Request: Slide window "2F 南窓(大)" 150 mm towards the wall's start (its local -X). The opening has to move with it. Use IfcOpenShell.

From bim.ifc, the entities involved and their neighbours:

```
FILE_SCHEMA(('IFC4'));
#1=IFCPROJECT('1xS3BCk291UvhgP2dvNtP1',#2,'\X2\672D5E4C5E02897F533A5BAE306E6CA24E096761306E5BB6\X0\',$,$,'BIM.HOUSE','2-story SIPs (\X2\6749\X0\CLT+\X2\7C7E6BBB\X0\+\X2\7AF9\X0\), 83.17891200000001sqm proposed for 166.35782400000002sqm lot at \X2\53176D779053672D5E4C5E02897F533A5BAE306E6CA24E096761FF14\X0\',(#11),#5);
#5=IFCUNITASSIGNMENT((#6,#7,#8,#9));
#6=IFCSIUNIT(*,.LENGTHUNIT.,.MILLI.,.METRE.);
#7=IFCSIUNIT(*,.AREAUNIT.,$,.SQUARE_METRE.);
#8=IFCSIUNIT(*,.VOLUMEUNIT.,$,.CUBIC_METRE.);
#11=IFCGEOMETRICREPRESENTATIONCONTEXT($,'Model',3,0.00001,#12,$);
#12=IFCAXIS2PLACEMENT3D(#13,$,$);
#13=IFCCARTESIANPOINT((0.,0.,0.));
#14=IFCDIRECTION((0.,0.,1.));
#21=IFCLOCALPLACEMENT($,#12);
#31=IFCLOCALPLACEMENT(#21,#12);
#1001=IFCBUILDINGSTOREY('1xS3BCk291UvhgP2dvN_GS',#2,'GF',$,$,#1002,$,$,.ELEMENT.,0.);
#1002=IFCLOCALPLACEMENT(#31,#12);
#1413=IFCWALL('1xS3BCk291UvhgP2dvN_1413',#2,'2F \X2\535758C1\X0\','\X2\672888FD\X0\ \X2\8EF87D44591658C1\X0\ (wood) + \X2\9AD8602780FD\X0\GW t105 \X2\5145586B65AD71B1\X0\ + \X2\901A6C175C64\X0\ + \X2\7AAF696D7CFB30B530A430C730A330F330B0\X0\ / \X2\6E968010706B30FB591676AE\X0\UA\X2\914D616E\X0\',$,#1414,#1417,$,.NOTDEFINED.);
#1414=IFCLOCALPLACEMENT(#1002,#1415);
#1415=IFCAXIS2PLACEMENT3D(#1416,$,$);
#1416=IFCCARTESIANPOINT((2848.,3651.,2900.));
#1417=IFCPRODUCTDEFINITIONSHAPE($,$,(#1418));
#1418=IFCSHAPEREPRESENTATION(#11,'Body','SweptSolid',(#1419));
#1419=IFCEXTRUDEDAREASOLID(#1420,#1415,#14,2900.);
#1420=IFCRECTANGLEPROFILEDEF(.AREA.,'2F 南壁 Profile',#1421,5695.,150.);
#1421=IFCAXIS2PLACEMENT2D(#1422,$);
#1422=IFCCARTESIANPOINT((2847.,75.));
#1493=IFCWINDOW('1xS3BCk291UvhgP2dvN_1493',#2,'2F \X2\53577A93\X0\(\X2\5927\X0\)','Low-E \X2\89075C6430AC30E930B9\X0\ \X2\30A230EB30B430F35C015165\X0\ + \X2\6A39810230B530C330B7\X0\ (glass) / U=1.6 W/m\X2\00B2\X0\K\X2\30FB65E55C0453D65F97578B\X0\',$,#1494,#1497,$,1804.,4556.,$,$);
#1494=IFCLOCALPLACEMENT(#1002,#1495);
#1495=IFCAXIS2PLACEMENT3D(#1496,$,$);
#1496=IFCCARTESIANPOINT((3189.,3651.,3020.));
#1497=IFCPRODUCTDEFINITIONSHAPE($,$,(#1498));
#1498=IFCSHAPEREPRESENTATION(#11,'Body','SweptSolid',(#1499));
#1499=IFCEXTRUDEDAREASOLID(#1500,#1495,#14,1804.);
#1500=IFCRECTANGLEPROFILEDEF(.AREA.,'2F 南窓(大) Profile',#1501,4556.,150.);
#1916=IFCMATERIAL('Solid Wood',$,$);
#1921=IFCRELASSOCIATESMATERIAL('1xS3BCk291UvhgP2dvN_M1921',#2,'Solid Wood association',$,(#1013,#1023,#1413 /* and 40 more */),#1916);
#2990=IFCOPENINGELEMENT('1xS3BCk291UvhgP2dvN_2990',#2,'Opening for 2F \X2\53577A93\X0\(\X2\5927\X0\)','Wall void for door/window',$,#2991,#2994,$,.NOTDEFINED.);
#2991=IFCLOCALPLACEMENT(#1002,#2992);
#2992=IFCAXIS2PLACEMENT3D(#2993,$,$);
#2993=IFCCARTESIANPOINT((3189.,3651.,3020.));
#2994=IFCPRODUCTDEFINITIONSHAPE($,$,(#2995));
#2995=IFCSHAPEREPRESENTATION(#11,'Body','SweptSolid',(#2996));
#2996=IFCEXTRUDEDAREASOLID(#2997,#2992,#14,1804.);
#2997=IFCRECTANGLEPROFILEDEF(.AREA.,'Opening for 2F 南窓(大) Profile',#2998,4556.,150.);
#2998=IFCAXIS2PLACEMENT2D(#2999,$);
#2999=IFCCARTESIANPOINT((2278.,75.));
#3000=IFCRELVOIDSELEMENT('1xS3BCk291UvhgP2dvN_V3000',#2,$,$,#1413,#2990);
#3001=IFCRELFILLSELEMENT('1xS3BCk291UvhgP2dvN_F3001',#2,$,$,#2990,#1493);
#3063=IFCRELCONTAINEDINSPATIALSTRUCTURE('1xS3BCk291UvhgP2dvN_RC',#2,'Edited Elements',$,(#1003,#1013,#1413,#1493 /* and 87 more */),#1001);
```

```python
import ifcopenshell
import ifcopenshell.api.geometry
import ifcopenshell.util.placement
import ifcopenshell.util.unit

model = ifcopenshell.open("bim.ifc")
unit_scale = ifcopenshell.util.unit.calculate_unit_scale(model)

window = model.by_guid("1xS3BCk291UvhgP2dvN_1493")
opening = window.FillsVoids[0].RelatingOpeningElement
wall = opening.VoidsElements[0].RelatingBuildingElement

wall_matrix = ifcopenshell.util.placement.get_local_placement(wall.ObjectPlacement)
shift = wall_matrix[:3, 0] * -0.15 / unit_scale
before = ifcopenshell.util.placement.get_local_placement(window.ObjectPlacement)[:3, 3].copy()

# The window is not placed relative to its opening, so move both.
for product in (opening, window):
    matrix = ifcopenshell.util.placement.get_local_placement(product.ObjectPlacement)
    matrix[:3, 3] += shift
    ifcopenshell.api.geometry.edit_object_placement(model, product=product, matrix=matrix, is_si=False)

after = ifcopenshell.util.placement.get_local_placement(window.ObjectPlacement)[:3, 3]
print("window moved by", (after - before).round(3) + 0.0)

model.write("bim_v2.ifc")
```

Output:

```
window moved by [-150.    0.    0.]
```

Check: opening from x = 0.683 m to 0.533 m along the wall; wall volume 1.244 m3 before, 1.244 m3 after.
